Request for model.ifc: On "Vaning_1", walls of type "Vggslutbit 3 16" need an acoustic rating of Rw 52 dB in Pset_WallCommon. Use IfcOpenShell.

First a look at what the model holds.

```python
import ifcopenshell
import ifcopenshell.util.element

model = ifcopenshell.open("model.ifc")
print(model.schema)
storey = next(s for s in model.by_type("IfcBuildingStorey") if s.Name == "Vaning_1")
walls = [e for e in ifcopenshell.util.element.get_decomposition(storey) if e.is_a("IfcWall")]
seen = {}
for e in walls:
    element_type = ifcopenshell.util.element.get_type(e)
    key = (element_type.Name if element_type != e and element_type else None, ifcopenshell.util.element.get_pset(e, "Pset_WallCommon", "AcousticRating"))
    seen[key] = seen.get(key, 0) + 1
for (name, value), count in sorted(seen.items(), key=str):
    print(count, "x", name, "|", value)
```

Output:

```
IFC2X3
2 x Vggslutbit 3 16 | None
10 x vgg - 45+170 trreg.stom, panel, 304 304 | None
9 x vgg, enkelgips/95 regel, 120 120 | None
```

```python
import ifcopenshell
import ifcopenshell.api.pset
import ifcopenshell.util.element

model = ifcopenshell.open("model.ifc")

storey = next(s for s in model.by_type("IfcBuildingStorey") if s.Name == "Vaning_1")
walls = [e for e in ifcopenshell.util.element.get_decomposition(storey) if e.is_a("IfcWall")]

count = 0
for e in walls:
    element_type = ifcopenshell.util.element.get_type(e)
    if element_type in (None, e) or element_type.Name != 'V\x8aggslutbit 3 16':
        continue
    # add_pset returns the element's existing set when there is one.
    pset = ifcopenshell.api.pset.add_pset(model, product=e, name="Pset_WallCommon")
    ifcopenshell.api.pset.edit_pset(model, pset=pset, properties={"AcousticRating": "Rw 52 dB"})
    count += 1

print(count, "walls updated")

model.write("model_updated.ifc")
```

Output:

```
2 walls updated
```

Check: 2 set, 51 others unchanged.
